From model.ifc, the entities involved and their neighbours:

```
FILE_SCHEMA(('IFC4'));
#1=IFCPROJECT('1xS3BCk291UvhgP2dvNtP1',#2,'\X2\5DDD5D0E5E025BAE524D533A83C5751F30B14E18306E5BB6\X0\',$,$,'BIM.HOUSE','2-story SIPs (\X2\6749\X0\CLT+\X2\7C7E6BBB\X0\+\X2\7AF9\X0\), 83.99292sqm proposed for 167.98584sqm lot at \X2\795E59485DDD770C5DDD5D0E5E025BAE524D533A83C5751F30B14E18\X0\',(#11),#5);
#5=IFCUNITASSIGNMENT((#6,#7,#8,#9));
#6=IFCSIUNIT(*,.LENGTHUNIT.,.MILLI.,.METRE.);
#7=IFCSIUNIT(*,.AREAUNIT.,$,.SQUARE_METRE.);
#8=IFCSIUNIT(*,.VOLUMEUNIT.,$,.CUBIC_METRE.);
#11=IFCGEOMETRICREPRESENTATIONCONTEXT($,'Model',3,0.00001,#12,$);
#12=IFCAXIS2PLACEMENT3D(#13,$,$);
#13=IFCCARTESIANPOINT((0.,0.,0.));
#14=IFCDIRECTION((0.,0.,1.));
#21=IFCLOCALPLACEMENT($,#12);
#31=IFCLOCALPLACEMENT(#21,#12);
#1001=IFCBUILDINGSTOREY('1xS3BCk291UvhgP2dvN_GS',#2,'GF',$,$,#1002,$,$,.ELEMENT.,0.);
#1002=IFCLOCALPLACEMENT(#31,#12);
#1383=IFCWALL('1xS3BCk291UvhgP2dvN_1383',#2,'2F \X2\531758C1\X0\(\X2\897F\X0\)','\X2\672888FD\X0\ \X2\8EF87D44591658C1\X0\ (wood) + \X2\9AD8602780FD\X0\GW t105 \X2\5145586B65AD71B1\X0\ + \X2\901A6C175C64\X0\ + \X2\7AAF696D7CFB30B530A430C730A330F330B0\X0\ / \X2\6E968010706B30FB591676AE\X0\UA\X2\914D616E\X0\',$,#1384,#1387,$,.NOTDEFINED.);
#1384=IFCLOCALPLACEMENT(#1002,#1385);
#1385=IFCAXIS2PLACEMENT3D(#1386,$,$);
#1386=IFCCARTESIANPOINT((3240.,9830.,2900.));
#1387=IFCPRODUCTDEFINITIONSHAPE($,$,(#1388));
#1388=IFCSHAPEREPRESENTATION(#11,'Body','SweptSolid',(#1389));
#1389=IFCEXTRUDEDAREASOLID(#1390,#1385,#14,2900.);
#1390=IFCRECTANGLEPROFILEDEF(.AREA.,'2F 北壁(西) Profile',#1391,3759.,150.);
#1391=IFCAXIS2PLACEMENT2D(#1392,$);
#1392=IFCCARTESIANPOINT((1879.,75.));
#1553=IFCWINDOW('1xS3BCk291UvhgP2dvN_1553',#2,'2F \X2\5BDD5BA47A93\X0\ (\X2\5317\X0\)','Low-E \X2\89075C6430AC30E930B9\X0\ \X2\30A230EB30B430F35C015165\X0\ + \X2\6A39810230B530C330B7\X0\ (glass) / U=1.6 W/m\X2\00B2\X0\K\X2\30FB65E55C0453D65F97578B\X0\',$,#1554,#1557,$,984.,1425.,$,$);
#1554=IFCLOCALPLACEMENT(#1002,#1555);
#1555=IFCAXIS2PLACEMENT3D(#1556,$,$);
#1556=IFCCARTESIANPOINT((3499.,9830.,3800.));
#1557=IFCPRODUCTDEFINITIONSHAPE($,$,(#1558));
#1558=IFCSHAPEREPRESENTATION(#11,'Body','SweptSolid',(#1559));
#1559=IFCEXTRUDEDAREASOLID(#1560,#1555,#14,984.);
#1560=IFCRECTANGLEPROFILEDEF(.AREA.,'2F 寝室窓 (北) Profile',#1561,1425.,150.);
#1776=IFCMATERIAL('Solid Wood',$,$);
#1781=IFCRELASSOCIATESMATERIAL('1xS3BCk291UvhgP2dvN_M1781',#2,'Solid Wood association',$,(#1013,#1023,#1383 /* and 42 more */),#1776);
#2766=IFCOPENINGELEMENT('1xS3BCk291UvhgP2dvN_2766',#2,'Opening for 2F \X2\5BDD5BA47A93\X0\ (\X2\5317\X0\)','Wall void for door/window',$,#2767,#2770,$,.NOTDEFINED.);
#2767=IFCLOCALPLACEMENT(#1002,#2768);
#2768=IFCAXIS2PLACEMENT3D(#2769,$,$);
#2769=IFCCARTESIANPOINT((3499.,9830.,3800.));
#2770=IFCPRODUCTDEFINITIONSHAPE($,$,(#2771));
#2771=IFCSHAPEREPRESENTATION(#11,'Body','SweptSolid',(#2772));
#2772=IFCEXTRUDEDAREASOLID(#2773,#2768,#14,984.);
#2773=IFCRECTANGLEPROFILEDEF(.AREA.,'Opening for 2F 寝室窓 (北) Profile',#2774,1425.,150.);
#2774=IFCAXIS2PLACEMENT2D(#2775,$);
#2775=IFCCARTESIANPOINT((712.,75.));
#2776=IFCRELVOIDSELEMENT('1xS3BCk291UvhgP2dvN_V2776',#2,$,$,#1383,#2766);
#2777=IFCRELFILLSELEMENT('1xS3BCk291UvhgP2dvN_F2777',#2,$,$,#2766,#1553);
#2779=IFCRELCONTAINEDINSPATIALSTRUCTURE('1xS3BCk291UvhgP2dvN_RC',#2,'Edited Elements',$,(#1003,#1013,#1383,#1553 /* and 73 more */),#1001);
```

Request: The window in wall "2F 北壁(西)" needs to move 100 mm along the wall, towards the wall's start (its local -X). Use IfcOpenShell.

```python
import ifcopenshell
import ifcopenshell.api.geometry
import ifcopenshell.util.placement
import ifcopenshell.util.unit

model = ifcopenshell.open("model.ifc")
unit_scale = ifcopenshell.util.unit.calculate_unit_scale(model)

window = model.by_guid("1xS3BCk291UvhgP2dvN_1553")
opening = window.FillsVoids[0].RelatingOpeningElement
wall = opening.VoidsElements[0].RelatingBuildingElement

wall_matrix = ifcopenshell.util.placement.get_local_placement(wall.ObjectPlacement)
shift = wall_matrix[:3, 0] * -0.1 / unit_scale
before = ifcopenshell.util.placement.get_local_placement(window.ObjectPlacement)[:3, 3].copy()

# The window is not placed relative to its opening, so move both.
for product in (opening, window):
    matrix = ifcopenshell.util.placement.get_local_placement(product.ObjectPlacement)
    matrix[:3, 3] += shift
    ifcopenshell.api.geometry.edit_object_placement(model, product=product, matrix=matrix, is_si=False)

after = ifcopenshell.util.placement.get_local_placement(window.ObjectPlacement)[:3, 3]
print("window moved by", (after - before).round(3) + 0.0)

model.write("model_updated.ifc")
```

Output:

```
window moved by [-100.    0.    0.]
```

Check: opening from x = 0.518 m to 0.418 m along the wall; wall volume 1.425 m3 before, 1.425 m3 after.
